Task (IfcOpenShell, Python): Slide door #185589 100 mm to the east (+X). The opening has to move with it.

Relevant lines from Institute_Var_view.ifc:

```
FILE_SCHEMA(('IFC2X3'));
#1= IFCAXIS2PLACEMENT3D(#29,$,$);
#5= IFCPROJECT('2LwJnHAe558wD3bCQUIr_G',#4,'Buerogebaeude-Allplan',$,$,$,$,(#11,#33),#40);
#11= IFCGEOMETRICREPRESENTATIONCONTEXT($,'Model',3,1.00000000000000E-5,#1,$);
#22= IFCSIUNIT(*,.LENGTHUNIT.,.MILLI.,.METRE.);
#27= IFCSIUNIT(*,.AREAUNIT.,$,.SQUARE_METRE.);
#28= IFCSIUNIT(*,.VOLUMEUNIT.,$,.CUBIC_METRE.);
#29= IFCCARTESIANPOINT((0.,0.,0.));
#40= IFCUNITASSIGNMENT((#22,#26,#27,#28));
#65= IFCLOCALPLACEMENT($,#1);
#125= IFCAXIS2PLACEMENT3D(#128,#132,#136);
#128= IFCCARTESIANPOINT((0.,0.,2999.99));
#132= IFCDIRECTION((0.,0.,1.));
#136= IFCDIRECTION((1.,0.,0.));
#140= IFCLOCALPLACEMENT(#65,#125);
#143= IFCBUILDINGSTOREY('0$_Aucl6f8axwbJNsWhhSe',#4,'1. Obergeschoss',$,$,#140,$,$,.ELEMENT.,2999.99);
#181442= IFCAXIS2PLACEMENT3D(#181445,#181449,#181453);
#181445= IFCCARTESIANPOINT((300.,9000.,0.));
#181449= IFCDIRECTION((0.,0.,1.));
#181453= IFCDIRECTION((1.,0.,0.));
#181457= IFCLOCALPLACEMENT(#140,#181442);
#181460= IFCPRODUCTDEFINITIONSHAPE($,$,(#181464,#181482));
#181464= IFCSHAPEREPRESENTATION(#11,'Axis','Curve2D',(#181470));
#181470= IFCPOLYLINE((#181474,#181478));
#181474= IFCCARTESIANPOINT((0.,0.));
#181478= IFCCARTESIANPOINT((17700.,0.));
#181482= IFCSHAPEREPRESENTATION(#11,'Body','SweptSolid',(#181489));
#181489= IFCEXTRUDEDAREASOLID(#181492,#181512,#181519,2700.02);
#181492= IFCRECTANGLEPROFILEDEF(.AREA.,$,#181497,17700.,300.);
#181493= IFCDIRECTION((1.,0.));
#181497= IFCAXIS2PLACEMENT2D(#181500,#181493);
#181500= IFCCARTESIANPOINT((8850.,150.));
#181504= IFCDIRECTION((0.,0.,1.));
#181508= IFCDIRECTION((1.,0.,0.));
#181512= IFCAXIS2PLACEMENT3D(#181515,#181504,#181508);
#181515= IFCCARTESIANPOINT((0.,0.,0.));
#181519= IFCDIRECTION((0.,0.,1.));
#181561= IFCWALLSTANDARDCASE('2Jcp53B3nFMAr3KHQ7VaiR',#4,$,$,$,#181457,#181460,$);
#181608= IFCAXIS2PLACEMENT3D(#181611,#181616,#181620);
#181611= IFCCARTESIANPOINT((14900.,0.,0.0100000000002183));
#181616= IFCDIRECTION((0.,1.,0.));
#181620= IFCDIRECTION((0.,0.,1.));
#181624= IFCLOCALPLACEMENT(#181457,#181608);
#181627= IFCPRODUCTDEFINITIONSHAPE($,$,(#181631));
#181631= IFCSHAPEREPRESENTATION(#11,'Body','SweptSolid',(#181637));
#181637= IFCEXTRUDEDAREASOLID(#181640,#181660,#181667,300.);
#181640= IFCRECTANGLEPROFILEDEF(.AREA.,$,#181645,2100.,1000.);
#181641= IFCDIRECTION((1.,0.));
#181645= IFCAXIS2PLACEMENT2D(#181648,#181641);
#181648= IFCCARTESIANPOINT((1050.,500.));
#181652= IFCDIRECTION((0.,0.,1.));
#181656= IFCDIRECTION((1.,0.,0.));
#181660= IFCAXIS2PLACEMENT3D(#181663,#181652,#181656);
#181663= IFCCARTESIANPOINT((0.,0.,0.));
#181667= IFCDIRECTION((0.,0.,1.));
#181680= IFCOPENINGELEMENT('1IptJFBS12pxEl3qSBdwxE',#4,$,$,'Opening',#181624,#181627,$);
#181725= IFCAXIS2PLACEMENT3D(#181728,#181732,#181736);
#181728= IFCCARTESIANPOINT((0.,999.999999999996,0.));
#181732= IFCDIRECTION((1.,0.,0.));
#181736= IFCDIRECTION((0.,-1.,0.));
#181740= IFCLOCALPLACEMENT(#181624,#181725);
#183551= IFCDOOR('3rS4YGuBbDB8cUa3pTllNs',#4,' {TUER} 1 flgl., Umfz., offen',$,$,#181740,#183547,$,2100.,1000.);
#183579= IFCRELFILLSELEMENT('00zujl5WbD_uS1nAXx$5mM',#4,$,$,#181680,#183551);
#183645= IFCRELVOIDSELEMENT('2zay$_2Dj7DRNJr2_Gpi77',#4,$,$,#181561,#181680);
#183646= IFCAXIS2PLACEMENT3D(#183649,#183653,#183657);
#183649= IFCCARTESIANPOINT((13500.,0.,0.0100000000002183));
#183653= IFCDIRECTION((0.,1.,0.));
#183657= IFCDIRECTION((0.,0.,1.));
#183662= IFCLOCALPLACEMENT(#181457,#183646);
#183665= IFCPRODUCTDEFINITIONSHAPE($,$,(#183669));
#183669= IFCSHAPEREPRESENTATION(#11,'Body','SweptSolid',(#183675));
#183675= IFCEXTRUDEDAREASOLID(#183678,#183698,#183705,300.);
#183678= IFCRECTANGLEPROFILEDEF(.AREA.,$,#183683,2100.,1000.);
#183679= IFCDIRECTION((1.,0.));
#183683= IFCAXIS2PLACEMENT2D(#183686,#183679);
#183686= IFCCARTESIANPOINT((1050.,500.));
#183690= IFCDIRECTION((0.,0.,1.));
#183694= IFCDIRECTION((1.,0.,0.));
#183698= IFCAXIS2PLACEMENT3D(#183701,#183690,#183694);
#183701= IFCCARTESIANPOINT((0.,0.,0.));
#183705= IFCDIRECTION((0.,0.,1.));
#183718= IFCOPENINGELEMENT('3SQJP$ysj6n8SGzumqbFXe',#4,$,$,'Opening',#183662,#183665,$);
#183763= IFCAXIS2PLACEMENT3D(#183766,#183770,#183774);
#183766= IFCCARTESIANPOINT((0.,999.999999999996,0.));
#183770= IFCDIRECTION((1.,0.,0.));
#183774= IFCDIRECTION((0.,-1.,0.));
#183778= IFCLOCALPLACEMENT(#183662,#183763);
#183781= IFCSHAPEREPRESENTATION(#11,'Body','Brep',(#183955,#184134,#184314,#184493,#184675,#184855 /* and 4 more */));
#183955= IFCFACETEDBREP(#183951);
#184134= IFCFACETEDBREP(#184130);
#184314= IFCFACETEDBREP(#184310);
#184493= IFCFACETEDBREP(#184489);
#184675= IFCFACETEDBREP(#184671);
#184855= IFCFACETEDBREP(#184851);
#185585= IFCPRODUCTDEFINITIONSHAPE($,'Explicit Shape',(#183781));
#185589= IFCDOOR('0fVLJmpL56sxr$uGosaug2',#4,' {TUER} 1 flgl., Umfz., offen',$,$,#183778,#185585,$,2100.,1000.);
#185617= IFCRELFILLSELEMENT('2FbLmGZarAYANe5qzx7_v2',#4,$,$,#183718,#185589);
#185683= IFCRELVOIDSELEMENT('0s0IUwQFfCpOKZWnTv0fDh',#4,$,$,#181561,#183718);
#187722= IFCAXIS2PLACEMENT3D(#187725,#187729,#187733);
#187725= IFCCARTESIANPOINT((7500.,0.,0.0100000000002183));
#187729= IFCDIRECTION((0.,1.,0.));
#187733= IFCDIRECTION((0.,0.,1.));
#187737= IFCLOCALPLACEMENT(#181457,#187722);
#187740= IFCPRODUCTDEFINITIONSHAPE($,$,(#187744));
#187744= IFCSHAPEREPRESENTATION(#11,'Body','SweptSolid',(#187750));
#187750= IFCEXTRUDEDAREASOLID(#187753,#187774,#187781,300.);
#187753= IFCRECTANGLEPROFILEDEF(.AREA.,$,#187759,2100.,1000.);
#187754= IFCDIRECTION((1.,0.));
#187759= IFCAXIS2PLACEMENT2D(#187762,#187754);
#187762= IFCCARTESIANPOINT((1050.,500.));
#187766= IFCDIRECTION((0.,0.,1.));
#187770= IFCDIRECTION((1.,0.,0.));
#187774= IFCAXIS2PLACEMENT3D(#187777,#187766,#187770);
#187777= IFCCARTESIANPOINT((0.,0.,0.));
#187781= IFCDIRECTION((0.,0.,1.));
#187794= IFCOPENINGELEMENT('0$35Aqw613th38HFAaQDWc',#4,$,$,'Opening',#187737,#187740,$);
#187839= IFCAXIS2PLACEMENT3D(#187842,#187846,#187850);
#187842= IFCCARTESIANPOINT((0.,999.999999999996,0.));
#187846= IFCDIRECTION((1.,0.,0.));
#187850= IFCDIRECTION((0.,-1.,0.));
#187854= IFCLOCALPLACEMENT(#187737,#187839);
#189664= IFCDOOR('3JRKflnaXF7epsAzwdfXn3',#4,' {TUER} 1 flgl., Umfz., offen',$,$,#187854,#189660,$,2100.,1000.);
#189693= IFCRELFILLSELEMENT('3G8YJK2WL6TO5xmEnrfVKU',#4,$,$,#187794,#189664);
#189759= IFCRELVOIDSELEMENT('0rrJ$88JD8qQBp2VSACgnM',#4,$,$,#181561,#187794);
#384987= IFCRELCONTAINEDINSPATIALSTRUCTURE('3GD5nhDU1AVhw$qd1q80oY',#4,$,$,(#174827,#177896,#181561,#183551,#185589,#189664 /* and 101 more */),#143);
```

```python
import ifcopenshell
import ifcopenshell.api.geometry
import ifcopenshell.util.placement
import ifcopenshell.util.unit

model = ifcopenshell.open("Institute_Var_view.ifc")
unit_scale = ifcopenshell.util.unit.calculate_unit_scale(model)

door = model.by_guid("0fVLJmpL56sxr$uGosaug2")
opening = door.FillsVoids[0].RelatingOpeningElement
wall = opening.VoidsElements[0].RelatingBuildingElement

wall_matrix = ifcopenshell.util.placement.get_local_placement(wall.ObjectPlacement)
shift = wall_matrix[:3, 0] * 0.1 / unit_scale
before = ifcopenshell.util.placement.get_local_placement(door.ObjectPlacement)[:3, 3].copy()

# The door is placed relative to its opening, so it follows when the opening moves.
matrix = ifcopenshell.util.placement.get_local_placement(opening.ObjectPlacement)
matrix[:3, 3] += shift
ifcopenshell.api.geometry.edit_object_placement(
    model, product=opening, matrix=matrix, is_si=False, should_transform_children=True
)

after = ifcopenshell.util.placement.get_local_placement(door.ObjectPlacement)[:3, 3]
print("door moved by", (after - before).round(3) + 0.0)

model.write("Institute_Var_view_v2.ifc")
```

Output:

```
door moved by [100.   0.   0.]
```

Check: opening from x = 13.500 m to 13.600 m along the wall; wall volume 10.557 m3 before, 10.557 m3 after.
